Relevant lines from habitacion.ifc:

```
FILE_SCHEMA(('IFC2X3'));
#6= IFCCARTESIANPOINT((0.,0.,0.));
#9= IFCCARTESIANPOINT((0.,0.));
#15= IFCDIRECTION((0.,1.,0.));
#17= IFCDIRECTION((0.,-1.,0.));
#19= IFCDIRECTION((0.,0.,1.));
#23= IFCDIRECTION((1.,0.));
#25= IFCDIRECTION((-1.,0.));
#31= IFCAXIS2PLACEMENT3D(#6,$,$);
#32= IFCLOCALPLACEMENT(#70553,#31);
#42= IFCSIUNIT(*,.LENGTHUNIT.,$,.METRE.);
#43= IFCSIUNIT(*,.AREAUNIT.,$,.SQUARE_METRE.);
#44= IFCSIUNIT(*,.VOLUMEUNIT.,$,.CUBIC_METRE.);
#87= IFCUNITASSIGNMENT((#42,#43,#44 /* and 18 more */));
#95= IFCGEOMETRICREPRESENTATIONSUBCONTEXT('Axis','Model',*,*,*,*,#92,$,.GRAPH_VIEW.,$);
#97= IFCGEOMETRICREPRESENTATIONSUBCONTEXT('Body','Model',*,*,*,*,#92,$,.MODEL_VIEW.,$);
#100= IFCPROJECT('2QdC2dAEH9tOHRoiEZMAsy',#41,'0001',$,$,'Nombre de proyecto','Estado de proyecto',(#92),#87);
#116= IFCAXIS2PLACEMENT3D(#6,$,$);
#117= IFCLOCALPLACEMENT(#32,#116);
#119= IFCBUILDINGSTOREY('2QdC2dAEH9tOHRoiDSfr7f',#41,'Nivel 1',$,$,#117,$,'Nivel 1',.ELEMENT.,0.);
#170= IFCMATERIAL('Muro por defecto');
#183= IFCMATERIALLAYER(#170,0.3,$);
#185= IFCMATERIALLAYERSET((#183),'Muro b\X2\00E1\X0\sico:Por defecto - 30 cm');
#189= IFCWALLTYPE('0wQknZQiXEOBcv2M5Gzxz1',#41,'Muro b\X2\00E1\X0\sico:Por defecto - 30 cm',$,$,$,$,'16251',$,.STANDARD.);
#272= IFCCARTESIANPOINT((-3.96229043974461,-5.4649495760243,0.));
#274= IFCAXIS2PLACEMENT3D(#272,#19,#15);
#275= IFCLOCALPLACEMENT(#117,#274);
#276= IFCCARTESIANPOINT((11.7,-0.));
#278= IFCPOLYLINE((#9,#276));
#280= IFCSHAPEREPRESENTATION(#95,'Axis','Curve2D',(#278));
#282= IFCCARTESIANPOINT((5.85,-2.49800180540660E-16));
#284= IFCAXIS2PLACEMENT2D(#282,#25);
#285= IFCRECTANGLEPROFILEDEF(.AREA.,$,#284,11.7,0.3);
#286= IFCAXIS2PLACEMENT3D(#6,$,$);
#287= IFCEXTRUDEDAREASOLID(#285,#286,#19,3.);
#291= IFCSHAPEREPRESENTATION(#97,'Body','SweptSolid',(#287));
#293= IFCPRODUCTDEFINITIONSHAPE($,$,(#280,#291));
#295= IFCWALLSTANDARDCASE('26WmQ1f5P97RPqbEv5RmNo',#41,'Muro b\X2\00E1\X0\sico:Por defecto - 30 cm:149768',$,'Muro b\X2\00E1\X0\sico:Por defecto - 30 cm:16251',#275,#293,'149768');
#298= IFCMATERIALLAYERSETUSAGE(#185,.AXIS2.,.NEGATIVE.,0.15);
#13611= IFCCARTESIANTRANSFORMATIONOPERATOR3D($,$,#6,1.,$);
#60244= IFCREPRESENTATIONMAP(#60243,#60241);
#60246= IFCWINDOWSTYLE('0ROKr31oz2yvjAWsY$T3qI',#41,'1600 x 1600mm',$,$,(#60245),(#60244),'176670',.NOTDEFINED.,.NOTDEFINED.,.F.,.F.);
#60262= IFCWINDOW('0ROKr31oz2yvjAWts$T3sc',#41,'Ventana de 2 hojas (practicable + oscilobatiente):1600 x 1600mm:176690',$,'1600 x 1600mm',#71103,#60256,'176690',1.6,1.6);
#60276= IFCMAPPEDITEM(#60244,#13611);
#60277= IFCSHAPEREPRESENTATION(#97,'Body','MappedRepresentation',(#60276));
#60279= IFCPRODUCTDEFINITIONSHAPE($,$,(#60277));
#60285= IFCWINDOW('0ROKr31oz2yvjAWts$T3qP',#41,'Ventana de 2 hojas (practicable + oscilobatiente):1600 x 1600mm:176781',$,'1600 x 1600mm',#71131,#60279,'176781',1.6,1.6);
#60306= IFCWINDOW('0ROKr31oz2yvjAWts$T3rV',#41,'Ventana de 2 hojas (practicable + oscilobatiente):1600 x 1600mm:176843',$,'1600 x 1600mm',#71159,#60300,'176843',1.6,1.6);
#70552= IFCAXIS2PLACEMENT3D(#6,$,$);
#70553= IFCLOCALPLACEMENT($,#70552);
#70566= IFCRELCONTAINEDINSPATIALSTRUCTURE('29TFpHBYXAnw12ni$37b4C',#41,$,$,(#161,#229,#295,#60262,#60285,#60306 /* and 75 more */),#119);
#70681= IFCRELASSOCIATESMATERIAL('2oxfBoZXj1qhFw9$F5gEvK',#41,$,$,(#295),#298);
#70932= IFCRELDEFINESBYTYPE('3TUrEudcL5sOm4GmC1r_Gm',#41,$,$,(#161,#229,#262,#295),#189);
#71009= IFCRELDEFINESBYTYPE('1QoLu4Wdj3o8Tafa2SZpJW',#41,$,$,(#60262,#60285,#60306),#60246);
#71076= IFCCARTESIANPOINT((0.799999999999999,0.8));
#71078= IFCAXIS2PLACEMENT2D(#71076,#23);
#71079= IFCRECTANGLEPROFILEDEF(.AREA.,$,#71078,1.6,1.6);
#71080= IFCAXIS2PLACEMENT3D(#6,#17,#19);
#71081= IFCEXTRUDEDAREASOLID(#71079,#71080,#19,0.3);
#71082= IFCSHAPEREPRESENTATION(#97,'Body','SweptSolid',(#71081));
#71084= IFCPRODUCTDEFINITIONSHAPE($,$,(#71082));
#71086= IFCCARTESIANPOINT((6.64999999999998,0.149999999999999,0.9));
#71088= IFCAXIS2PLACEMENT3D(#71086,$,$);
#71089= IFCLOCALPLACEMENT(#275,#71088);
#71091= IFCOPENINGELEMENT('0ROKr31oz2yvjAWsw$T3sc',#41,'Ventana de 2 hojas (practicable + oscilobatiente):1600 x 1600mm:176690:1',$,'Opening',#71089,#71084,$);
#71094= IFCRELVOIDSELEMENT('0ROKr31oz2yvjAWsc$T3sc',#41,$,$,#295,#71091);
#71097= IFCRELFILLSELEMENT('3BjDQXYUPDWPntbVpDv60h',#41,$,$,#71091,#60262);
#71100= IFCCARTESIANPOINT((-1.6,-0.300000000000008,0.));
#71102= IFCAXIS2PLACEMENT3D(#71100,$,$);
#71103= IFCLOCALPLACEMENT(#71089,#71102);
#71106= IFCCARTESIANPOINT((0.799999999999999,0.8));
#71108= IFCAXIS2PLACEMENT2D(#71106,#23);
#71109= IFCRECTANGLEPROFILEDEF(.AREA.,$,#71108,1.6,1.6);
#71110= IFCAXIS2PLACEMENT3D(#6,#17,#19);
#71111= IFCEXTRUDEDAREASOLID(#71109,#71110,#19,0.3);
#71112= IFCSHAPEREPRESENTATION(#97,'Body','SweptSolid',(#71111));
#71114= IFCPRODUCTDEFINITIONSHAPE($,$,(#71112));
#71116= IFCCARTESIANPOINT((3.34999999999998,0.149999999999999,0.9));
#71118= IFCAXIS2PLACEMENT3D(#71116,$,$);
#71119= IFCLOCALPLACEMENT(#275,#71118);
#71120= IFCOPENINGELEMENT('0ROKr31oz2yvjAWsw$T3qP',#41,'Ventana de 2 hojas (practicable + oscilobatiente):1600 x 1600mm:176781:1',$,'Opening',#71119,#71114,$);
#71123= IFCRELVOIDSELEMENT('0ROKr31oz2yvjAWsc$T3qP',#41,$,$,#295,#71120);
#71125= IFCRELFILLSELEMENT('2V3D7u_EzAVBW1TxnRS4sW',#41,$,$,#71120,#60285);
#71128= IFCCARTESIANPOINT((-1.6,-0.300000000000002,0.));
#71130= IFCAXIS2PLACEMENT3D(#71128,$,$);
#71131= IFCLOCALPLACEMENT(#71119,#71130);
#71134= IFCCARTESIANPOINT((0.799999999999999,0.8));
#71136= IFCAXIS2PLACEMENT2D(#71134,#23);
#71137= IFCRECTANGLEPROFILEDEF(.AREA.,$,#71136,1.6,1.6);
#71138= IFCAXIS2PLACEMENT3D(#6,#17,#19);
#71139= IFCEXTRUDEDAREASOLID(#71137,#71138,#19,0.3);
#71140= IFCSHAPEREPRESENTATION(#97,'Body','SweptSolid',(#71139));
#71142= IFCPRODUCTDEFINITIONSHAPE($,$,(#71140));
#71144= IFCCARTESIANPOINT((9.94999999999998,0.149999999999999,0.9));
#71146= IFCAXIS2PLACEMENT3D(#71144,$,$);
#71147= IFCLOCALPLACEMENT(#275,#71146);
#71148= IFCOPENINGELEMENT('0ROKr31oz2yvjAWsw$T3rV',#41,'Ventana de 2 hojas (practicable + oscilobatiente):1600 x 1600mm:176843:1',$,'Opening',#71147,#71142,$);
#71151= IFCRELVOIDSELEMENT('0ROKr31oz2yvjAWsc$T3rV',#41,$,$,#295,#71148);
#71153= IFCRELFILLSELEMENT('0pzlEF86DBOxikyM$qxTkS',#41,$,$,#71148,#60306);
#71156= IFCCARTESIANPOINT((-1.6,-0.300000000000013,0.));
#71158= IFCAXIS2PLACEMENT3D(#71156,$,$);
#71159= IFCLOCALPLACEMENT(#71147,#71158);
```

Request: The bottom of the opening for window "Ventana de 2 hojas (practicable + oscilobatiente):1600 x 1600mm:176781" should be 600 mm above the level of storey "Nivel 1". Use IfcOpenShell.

```python
import numpy as np
import ifcopenshell
import ifcopenshell.api.geometry
import ifcopenshell.geom
import ifcopenshell.util.element
import ifcopenshell.util.placement
import ifcopenshell.util.shape
import ifcopenshell.util.unit

model = ifcopenshell.open("habitacion.ifc")
unit_scale = ifcopenshell.util.unit.calculate_unit_scale(model)

window = model.by_guid("0ROKr31oz2yvjAWts$T3qP")
opening = window.FillsVoids[0].RelatingOpeningElement
storey = ifcopenshell.util.element.get_container(window, ifc_class="IfcBuildingStorey")
level = ifcopenshell.util.placement.get_local_placement(storey.ObjectPlacement)[2, 3]

# The opening's origin need not be at the sill, so measure its lowest point.
shape = ifcopenshell.geom.create_shape(ifcopenshell.geom.settings(), opening)
bottom = ifcopenshell.util.shape.get_shape_bottom_elevation(shape, shape.geometry) / unit_scale
dz = level + 0.6 - bottom

shift = np.array([0.0, 0.0, dz])
# The window is placed relative to its opening, so it follows when the opening moves.
matrix = ifcopenshell.util.placement.get_local_placement(opening.ObjectPlacement)
matrix[:3, 3] += shift
ifcopenshell.api.geometry.edit_object_placement(
    model, product=opening, matrix=matrix, is_si=False, should_transform_children=True
)

print(f"moved by {dz * unit_scale:+.3f} m")

model.write("habitacion_rev.ifc")
```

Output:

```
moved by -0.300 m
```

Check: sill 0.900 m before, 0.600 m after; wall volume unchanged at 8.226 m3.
